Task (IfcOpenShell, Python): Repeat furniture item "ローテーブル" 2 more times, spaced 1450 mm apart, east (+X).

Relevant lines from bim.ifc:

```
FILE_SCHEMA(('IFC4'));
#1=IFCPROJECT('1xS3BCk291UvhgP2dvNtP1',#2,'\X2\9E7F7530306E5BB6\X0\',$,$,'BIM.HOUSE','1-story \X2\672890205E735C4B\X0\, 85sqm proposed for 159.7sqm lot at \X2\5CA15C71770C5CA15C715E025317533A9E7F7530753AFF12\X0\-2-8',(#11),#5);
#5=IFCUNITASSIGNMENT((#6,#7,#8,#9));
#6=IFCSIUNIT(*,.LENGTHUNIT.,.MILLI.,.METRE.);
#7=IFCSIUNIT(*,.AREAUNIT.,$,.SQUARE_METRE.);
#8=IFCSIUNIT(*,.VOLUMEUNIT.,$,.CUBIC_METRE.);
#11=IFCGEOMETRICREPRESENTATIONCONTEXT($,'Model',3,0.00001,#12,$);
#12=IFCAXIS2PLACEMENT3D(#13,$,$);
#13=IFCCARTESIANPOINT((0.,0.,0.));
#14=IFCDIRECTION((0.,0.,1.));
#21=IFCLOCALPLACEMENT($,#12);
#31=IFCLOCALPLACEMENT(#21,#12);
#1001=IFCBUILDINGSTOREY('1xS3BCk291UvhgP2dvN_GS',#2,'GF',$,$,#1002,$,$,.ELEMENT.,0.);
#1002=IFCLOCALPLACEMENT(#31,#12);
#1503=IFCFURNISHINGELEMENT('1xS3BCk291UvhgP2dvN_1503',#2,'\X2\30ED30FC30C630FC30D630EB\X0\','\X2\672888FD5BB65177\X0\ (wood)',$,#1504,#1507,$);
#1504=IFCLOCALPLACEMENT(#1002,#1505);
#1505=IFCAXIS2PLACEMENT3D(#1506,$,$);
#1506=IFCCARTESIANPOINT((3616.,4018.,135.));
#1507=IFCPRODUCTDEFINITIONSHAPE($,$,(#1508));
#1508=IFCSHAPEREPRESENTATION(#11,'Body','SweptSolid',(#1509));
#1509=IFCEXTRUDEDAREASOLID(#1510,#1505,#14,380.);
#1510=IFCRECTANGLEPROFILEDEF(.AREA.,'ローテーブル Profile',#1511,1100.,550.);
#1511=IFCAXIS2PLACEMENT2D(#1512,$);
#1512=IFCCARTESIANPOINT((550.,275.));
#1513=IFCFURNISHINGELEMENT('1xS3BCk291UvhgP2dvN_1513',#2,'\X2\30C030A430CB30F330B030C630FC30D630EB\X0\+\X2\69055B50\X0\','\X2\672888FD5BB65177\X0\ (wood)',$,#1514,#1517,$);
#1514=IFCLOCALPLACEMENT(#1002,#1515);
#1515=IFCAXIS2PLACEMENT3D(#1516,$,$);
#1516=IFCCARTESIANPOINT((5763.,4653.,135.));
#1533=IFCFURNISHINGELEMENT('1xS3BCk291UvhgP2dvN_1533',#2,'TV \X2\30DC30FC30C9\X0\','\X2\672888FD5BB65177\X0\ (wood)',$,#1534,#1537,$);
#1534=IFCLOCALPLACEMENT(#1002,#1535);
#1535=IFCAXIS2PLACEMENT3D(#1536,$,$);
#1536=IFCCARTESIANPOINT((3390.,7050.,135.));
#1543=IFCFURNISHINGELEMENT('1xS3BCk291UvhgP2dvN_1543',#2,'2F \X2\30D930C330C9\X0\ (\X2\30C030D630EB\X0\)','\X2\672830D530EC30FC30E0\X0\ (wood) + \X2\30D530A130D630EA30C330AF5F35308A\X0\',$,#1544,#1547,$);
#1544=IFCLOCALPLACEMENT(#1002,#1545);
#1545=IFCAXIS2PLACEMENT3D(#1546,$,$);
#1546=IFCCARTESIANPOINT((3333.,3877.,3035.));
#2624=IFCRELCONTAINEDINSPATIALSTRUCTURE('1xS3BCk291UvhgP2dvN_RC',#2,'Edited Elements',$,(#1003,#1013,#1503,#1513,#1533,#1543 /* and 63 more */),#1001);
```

```python
import numpy as np
import ifcopenshell
import ifcopenshell.api.geometry
import ifcopenshell.api.root
import ifcopenshell.util.element
import ifcopenshell.util.placement

model = ifcopenshell.open("bim.ifc")


def reuse_history(source, copy):
    """copy_class also copies each property set's owner history, people and application; keep the originals."""
    for rel in copy.IsDefinedBy:
        if rel.is_a("IfcRelDefinesByProperties") and (history := rel.RelatingPropertyDefinition.OwnerHistory):
            rel.RelatingPropertyDefinition.OwnerHistory = source.OwnerHistory
            ifcopenshell.util.element.remove_deep2(model, history)


source = model.by_id(1503)
base = ifcopenshell.util.placement.get_local_placement(source.ObjectPlacement)
step = np.array([1.0, 0.0, 0.0]) * 1450.0

for i in range(1, 3):
    copy = ifcopenshell.api.root.copy_class(model, product=source)
    copy.Representation = ifcopenshell.util.element.copy_deep(
        model, source.Representation, exclude=["IfcGeometricRepresentationContext", "IfcRepresentationMap"]
    )
    reuse_history(source, copy)
    matrix = base.copy()
    matrix[:3, 3] += i * step
    print("added at", matrix[:3, 3].round(3) + 0.0)
    ifcopenshell.api.geometry.edit_object_placement(model, product=copy, matrix=matrix, is_si=False)

model.write("bim_v2.ifc")
```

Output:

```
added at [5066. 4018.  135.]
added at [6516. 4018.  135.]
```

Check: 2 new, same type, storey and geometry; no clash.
